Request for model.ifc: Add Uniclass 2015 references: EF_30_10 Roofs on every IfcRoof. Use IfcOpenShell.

First a look at what the model holds.

```python
import ifcopenshell

model = ifcopenshell.open("model.ifc")
print(model.schema)
print("classifications:", [c.Name for c in model.by_type("IfcClassification")])
for ifc_class in ("IfcDoor", "IfcRoof", "IfcStair", "IfcWall", "IfcWindow"):
    print(ifc_class, len(model.by_type(ifc_class)))
```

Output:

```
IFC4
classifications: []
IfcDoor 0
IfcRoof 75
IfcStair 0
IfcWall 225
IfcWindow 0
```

```python
import ifcopenshell
import ifcopenshell.api.classification

model = ifcopenshell.open("model.ifc")

system = ifcopenshell.api.classification.add_classification(model, classification="Uniclass 2015")

codes = {
    "IfcRoof": ("EF_30_10", "Roofs"),
}
for ifc_class, (code, name) in codes.items():
    products = model.by_type(ifc_class)
    ifcopenshell.api.classification.add_reference(
        model, products=products, classification=system, identification=code, name=name
    )
    print(code, len(products))

model.write("model-out.ifc")
```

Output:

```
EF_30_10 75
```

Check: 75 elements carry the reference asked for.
